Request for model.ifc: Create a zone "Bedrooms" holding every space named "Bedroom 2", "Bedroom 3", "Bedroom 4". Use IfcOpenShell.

First a look at what the model holds.

```python
import ifcopenshell

model = ifcopenshell.open("model.ifc")
print(model.schema)
seen = {}
for space in model.by_type("IfcSpace"):
    seen[space.LongName] = seen.get(space.LongName, 0) + 1
for name, count in sorted(seen.items(), key=str):
    print(count, "x", name)
print("zones:", [z.Name for z in model.by_type("IfcZone")][:20])
```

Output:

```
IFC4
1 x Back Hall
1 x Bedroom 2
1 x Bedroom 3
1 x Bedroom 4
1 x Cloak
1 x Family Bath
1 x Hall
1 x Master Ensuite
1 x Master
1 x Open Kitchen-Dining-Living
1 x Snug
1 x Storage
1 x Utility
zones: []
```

```python
import ifcopenshell
import ifcopenshell.api.group
import ifcopenshell.api.root

model = ifcopenshell.open("model.ifc")

names = {"Bedroom 2", "Bedroom 3", "Bedroom 4"}
spaces = [s for s in model.by_type("IfcSpace") if s.LongName in names]

zone = ifcopenshell.api.root.create_entity(model, ifc_class="IfcZone", name="Bedrooms")
ifcopenshell.api.group.assign_group(model, products=spaces, group=zone)
print(len(spaces), "spaces in", zone.Name)

model.write("model_v2.ifc")
```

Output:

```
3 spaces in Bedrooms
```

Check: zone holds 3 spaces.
